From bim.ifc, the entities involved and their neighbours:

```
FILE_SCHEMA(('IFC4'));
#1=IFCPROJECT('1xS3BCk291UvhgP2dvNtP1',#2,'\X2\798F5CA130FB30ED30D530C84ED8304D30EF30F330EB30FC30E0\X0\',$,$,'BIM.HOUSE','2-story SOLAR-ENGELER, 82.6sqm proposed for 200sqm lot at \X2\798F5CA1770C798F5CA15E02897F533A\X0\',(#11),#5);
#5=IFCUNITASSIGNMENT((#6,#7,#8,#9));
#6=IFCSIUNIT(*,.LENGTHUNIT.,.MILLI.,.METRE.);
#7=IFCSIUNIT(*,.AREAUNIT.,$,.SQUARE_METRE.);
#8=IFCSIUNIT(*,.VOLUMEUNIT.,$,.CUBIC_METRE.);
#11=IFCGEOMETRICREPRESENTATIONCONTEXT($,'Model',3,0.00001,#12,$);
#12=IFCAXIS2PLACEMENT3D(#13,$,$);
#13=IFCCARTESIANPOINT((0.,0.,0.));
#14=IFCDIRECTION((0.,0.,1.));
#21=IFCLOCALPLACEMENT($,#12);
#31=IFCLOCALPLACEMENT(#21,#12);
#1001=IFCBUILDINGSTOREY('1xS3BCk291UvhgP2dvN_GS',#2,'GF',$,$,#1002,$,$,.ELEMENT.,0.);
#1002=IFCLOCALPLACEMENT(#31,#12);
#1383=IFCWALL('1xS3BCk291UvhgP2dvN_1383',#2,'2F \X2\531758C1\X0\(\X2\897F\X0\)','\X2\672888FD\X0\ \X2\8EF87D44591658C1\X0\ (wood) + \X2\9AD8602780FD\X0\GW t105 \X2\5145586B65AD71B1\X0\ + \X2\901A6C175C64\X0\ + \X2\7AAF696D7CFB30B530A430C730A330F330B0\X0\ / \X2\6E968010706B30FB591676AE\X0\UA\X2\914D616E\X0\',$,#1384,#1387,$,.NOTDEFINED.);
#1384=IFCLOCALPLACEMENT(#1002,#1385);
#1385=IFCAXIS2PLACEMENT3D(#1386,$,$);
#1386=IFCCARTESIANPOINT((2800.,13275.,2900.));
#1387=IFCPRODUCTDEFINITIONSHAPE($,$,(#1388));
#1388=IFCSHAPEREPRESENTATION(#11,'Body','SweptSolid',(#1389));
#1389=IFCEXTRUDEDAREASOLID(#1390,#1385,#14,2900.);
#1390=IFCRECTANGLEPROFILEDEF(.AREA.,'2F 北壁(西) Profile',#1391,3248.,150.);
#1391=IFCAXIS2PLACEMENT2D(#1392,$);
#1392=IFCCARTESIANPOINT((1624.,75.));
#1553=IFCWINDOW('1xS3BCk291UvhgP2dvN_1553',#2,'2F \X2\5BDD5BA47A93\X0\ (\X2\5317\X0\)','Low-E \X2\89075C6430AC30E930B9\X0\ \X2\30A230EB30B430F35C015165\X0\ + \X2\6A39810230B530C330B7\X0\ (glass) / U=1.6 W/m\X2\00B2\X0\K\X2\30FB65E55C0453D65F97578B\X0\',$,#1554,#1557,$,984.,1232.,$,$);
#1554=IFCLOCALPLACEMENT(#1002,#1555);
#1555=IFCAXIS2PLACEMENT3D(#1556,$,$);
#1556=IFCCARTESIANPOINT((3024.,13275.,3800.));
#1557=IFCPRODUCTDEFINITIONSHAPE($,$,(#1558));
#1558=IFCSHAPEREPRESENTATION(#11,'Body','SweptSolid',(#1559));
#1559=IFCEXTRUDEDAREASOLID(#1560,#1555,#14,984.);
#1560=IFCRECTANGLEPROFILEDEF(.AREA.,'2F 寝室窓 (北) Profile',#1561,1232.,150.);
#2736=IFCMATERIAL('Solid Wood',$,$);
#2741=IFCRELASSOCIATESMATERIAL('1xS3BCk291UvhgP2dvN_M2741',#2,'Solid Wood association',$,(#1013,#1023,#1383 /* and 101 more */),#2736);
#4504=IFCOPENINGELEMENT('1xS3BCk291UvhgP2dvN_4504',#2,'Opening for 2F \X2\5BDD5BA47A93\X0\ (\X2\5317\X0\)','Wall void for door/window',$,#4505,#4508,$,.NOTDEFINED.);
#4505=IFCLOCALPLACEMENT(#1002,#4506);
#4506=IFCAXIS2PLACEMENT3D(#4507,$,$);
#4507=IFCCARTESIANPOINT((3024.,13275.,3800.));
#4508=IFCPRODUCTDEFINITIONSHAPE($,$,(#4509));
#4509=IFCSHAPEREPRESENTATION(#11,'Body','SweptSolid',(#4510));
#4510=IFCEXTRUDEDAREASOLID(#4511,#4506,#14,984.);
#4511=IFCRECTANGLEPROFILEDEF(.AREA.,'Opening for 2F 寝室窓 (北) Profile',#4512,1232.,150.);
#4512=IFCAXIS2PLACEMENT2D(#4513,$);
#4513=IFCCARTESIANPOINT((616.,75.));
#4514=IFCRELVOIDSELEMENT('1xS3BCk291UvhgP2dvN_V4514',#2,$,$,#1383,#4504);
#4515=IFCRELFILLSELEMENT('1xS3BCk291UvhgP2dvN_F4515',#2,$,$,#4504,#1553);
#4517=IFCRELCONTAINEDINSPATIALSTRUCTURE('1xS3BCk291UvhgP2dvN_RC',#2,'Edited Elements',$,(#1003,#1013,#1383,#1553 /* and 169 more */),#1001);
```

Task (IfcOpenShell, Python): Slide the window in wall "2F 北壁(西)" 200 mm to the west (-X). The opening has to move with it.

```python
import ifcopenshell
import ifcopenshell.api.geometry
import ifcopenshell.util.placement

model = ifcopenshell.open("bim.ifc")

window = model.by_id(1553)
opening = window.FillsVoids[0].RelatingOpeningElement
wall = opening.VoidsElements[0].RelatingBuildingElement

wall_matrix = ifcopenshell.util.placement.get_local_placement(wall.ObjectPlacement)
shift = wall_matrix[:3, 0] * -200.0
before = ifcopenshell.util.placement.get_local_placement(window.ObjectPlacement)[:3, 3].copy()

# The window is not placed relative to its opening, so move both.
for product in (opening, window):
    matrix = ifcopenshell.util.placement.get_local_placement(product.ObjectPlacement)
    matrix[:3, 3] += shift
    ifcopenshell.api.geometry.edit_object_placement(model, product=product, matrix=matrix, is_si=False)

after = ifcopenshell.util.placement.get_local_placement(window.ObjectPlacement)[:3, 3]
print("window moved by", (after - before).round(3) + 0.0)

model.write("bim_rev.ifc")
```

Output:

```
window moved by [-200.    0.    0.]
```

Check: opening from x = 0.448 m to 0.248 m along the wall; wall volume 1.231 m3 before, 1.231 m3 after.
